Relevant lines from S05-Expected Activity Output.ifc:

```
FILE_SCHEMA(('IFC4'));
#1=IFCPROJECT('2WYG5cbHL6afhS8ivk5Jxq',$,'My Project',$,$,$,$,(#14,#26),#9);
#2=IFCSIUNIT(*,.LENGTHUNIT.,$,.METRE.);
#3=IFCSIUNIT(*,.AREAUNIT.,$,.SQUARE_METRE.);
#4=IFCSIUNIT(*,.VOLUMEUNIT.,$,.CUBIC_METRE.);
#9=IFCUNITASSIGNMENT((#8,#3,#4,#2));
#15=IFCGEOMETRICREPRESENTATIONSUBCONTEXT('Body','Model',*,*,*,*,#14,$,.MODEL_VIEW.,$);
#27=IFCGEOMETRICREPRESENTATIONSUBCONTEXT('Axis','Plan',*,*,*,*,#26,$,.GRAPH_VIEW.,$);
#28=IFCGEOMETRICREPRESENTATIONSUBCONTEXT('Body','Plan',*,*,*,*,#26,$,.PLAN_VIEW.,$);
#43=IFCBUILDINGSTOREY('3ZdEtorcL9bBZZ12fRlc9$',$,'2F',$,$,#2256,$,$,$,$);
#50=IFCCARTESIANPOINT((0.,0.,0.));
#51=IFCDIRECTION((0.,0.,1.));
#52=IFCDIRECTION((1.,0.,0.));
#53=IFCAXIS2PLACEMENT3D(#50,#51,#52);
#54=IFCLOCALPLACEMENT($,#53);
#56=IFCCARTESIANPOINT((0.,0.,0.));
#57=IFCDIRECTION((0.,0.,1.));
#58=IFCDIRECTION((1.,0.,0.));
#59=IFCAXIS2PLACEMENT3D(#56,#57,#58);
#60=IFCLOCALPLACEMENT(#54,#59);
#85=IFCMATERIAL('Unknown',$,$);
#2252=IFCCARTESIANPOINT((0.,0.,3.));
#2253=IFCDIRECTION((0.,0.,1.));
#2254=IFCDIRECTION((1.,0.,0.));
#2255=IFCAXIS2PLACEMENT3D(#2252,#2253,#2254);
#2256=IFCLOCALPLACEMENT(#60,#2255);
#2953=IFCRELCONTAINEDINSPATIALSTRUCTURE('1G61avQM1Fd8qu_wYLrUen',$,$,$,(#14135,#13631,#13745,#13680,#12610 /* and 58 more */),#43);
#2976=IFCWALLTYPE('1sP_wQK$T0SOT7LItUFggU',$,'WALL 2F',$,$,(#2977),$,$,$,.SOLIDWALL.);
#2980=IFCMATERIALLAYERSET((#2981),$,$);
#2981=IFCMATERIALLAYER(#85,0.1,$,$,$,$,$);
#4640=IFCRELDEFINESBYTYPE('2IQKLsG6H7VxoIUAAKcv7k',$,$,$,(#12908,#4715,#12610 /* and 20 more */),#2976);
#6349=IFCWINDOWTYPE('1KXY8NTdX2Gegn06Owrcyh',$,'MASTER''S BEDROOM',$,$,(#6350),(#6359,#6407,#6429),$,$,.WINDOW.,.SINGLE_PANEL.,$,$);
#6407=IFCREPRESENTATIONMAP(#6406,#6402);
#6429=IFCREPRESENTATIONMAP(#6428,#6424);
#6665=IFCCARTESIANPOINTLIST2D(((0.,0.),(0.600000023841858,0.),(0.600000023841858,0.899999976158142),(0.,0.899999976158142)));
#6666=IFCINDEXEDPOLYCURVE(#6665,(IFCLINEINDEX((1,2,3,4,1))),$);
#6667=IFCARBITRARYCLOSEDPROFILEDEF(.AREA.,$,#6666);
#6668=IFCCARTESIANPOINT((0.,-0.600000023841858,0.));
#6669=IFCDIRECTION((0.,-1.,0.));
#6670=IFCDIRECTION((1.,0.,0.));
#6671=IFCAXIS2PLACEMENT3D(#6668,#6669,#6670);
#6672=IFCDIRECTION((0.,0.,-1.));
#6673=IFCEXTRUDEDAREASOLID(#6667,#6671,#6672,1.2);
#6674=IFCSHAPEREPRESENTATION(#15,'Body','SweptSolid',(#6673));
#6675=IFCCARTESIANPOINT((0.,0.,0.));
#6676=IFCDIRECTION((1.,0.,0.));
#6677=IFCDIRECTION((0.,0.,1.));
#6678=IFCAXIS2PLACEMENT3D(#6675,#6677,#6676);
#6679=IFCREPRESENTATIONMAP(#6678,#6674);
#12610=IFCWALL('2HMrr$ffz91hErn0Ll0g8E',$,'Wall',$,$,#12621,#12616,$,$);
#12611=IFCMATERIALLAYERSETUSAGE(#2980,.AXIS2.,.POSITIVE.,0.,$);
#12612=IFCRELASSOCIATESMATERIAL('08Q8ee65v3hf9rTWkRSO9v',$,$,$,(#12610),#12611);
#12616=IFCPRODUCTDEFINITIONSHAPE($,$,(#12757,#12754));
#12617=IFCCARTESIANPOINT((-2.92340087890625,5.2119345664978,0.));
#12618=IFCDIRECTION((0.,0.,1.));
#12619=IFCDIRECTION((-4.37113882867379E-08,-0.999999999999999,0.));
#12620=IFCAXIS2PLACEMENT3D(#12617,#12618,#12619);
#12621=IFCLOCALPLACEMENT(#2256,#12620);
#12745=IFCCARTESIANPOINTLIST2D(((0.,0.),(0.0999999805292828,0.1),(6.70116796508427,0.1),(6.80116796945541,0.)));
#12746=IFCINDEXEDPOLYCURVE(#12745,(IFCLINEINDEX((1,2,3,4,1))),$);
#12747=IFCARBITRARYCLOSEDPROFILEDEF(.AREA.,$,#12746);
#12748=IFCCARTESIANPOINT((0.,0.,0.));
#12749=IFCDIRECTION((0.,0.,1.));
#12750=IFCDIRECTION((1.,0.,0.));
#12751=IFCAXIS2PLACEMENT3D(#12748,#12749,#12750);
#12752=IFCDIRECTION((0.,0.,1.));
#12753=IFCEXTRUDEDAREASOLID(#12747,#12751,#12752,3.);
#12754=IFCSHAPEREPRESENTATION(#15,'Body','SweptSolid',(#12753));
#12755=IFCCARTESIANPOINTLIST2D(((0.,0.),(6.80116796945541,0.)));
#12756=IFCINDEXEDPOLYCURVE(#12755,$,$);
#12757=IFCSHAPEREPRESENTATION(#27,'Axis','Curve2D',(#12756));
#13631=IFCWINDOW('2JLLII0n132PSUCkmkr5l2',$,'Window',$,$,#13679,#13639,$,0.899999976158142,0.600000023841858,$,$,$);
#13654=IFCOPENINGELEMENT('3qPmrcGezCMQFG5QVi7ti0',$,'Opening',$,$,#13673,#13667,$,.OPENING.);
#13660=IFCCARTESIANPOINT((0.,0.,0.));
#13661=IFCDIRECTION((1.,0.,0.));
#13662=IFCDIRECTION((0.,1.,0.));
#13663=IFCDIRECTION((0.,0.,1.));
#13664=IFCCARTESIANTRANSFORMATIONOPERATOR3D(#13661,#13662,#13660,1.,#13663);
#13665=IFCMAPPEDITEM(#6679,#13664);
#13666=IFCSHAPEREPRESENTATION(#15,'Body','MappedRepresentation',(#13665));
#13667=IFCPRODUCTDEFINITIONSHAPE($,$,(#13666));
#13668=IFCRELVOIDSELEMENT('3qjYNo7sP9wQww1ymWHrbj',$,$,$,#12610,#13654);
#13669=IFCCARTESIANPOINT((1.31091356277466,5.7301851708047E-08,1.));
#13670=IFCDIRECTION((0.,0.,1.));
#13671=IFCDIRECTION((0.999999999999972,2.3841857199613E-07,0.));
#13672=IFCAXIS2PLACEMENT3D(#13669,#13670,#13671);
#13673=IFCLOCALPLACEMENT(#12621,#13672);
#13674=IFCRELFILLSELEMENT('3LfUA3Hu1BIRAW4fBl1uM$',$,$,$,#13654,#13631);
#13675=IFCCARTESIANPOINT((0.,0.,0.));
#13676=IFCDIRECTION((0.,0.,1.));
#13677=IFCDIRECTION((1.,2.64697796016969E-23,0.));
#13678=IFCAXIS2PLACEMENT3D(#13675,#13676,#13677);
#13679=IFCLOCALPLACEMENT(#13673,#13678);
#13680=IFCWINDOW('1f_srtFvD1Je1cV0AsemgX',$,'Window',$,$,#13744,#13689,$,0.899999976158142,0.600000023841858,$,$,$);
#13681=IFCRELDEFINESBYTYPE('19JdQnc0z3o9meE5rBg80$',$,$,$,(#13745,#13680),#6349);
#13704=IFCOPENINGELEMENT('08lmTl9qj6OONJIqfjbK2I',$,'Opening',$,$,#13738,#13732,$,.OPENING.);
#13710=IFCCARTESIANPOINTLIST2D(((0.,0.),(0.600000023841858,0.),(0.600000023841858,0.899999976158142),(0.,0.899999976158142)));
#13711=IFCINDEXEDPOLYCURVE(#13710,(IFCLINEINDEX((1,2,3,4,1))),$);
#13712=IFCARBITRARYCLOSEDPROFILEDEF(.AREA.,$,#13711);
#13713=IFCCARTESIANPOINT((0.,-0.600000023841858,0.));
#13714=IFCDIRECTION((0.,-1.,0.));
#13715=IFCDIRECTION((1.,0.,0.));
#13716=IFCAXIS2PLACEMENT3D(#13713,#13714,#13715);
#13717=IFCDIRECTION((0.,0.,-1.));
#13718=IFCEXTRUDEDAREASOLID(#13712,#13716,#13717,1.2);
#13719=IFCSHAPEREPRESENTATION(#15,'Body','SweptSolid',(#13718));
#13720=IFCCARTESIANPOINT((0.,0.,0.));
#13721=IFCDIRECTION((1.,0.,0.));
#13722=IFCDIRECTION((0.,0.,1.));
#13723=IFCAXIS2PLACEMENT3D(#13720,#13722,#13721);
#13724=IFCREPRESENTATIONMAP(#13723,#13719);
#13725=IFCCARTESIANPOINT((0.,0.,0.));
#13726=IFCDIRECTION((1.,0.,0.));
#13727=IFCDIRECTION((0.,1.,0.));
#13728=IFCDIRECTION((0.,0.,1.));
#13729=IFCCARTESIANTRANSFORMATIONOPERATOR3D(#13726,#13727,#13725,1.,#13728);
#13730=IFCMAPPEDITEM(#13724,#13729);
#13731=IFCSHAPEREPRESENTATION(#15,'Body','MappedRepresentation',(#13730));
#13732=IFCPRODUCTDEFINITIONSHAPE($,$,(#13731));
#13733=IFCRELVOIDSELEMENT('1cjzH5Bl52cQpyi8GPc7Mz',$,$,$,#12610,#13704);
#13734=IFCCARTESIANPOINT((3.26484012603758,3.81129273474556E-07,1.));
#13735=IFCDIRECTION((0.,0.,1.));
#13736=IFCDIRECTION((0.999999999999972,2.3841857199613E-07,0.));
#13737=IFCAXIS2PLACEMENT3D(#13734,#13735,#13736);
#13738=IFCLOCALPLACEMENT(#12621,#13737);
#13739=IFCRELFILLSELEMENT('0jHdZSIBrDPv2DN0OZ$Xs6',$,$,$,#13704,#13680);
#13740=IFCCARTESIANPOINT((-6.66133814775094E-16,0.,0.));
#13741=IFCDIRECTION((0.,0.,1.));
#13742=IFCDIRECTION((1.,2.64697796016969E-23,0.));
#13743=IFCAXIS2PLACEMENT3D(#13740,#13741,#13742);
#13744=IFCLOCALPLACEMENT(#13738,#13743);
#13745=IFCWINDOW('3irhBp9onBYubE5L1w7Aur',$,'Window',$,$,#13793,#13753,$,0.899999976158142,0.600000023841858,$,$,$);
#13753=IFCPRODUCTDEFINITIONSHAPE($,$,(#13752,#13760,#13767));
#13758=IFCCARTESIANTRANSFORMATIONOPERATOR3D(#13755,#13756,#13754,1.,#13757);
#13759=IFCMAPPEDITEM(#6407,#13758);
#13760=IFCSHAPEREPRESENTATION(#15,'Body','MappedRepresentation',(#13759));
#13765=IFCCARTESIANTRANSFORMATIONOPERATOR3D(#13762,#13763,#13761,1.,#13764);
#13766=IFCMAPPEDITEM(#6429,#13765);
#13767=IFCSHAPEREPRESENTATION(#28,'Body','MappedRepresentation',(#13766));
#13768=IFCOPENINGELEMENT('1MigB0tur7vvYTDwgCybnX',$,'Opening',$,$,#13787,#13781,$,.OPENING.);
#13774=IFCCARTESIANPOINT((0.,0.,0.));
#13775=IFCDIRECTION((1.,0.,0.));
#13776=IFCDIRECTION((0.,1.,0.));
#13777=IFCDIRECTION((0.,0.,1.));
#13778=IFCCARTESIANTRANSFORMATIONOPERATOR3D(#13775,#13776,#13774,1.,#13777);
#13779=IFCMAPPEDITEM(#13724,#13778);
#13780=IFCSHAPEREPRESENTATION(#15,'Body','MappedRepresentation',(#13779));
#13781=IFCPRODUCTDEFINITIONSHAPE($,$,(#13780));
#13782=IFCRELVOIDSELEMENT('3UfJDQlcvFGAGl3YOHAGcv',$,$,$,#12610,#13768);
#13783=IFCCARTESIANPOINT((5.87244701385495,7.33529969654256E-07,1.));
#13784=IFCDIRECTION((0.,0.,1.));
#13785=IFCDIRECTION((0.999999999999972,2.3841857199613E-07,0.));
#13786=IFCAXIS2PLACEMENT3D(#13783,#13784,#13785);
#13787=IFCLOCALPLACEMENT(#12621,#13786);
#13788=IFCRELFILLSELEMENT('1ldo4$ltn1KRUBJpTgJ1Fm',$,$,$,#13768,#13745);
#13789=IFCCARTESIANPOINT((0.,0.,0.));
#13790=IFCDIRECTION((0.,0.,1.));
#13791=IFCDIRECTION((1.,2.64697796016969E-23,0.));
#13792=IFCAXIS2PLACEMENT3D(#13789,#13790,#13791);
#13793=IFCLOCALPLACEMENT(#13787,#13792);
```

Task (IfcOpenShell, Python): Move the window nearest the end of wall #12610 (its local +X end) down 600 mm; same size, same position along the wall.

```python
import numpy as np
import ifcopenshell
import ifcopenshell.api.geometry
import ifcopenshell.util.placement
import ifcopenshell.util.unit

model = ifcopenshell.open("S05-Expected Activity Output.ifc")
unit_scale = ifcopenshell.util.unit.calculate_unit_scale(model)

window = model.by_id(13745)
opening = window.FillsVoids[0].RelatingOpeningElement
dz = -0.6 / unit_scale

shift = np.array([0.0, 0.0, dz])
# The window is placed relative to its opening, so it follows when the opening moves.
matrix = ifcopenshell.util.placement.get_local_placement(opening.ObjectPlacement)
matrix[:3, 3] += shift
ifcopenshell.api.geometry.edit_object_placement(
    model, product=opening, matrix=matrix, is_si=False, should_transform_children=True
)

print(f"moved by {dz * unit_scale:+.3f} m")

model.write("S05-Expected Activity Output_v2.ifc")
```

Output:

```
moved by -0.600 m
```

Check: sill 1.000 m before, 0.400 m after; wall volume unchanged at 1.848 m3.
